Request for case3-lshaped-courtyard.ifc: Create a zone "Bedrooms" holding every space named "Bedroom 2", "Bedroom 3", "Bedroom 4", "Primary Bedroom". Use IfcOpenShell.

First a look at what the model holds.

```python
import ifcopenshell

model = ifcopenshell.open("case3-lshaped-courtyard.ifc")
print(model.schema)
seen = {}
for space in model.by_type("IfcSpace"):
    seen[space.Name] = seen.get(space.Name, 0) + 1
for name, count in sorted(seen.items(), key=str):
    print(count, "x", name)
print("zones:", [z.Name for z in model.by_type("IfcZone")][:20])
```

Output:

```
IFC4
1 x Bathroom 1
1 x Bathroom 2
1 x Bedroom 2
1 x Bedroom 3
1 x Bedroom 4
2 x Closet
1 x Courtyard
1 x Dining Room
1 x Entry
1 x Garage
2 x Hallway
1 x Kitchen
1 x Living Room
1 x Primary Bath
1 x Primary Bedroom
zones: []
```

```python
import ifcopenshell
import ifcopenshell.api.group
import ifcopenshell.api.root

model = ifcopenshell.open("case3-lshaped-courtyard.ifc")

names = {"Bedroom 2", "Bedroom 3", "Bedroom 4", "Primary Bedroom"}
spaces = [s for s in model.by_type("IfcSpace") if s.Name in names]

zone = ifcopenshell.api.root.create_entity(model, ifc_class="IfcZone", name="Bedrooms")
ifcopenshell.api.group.assign_group(model, products=spaces, group=zone)
print(len(spaces), "spaces in", zone.Name)

model.write("case3-lshaped-courtyard_v2.ifc")
```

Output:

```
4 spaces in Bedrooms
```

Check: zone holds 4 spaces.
